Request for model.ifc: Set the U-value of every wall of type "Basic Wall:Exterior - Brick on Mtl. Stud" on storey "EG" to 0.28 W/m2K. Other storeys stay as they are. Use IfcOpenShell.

First a look at what the model holds.

```python
import ifcopenshell
import ifcopenshell.util.element

model = ifcopenshell.open("model.ifc")
print(model.schema)
storey = next(s for s in model.by_type("IfcBuildingStorey") if s.Name == "EG")
walls = [e for e in ifcopenshell.util.element.get_decomposition(storey) if e.is_a("IfcWall")]
seen = {}
for e in walls:
    element_type = ifcopenshell.util.element.get_type(e)
    key = (element_type.Name if element_type != e and element_type else None, ifcopenshell.util.element.get_pset(e, "Pset_WallCommon", "ThermalTransmittance"))
    seen[key] = seen.get(key, 0) + 1
for (name, value), count in sorted(seen.items(), key=str):
    print(count, "x", name, "|", value)
```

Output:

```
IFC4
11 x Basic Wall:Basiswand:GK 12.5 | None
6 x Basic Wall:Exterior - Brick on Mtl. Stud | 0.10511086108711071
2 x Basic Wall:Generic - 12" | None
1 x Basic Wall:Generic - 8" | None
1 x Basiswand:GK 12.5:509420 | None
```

```python
import ifcopenshell
import ifcopenshell.api.pset
import ifcopenshell.util.element

model = ifcopenshell.open("model.ifc")

storey = next(s for s in model.by_type("IfcBuildingStorey") if s.Name == "EG")
walls = [e for e in ifcopenshell.util.element.get_decomposition(storey) if e.is_a("IfcWall")]

count = 0
for e in walls:
    element_type = ifcopenshell.util.element.get_type(e)
    if element_type in (None, e) or element_type.Name != "Basic Wall:Exterior - Brick on Mtl. Stud":
        continue
    # add_pset returns the element's existing set when there is one.
    pset = ifcopenshell.api.pset.add_pset(model, product=e, name="Pset_WallCommon")
    ifcopenshell.api.pset.edit_pset(model, pset=pset, properties={"ThermalTransmittance": 0.28})
    count += 1

print(count, "walls updated")

model.write("model_rev.ifc")
```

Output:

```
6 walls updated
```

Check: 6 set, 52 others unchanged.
